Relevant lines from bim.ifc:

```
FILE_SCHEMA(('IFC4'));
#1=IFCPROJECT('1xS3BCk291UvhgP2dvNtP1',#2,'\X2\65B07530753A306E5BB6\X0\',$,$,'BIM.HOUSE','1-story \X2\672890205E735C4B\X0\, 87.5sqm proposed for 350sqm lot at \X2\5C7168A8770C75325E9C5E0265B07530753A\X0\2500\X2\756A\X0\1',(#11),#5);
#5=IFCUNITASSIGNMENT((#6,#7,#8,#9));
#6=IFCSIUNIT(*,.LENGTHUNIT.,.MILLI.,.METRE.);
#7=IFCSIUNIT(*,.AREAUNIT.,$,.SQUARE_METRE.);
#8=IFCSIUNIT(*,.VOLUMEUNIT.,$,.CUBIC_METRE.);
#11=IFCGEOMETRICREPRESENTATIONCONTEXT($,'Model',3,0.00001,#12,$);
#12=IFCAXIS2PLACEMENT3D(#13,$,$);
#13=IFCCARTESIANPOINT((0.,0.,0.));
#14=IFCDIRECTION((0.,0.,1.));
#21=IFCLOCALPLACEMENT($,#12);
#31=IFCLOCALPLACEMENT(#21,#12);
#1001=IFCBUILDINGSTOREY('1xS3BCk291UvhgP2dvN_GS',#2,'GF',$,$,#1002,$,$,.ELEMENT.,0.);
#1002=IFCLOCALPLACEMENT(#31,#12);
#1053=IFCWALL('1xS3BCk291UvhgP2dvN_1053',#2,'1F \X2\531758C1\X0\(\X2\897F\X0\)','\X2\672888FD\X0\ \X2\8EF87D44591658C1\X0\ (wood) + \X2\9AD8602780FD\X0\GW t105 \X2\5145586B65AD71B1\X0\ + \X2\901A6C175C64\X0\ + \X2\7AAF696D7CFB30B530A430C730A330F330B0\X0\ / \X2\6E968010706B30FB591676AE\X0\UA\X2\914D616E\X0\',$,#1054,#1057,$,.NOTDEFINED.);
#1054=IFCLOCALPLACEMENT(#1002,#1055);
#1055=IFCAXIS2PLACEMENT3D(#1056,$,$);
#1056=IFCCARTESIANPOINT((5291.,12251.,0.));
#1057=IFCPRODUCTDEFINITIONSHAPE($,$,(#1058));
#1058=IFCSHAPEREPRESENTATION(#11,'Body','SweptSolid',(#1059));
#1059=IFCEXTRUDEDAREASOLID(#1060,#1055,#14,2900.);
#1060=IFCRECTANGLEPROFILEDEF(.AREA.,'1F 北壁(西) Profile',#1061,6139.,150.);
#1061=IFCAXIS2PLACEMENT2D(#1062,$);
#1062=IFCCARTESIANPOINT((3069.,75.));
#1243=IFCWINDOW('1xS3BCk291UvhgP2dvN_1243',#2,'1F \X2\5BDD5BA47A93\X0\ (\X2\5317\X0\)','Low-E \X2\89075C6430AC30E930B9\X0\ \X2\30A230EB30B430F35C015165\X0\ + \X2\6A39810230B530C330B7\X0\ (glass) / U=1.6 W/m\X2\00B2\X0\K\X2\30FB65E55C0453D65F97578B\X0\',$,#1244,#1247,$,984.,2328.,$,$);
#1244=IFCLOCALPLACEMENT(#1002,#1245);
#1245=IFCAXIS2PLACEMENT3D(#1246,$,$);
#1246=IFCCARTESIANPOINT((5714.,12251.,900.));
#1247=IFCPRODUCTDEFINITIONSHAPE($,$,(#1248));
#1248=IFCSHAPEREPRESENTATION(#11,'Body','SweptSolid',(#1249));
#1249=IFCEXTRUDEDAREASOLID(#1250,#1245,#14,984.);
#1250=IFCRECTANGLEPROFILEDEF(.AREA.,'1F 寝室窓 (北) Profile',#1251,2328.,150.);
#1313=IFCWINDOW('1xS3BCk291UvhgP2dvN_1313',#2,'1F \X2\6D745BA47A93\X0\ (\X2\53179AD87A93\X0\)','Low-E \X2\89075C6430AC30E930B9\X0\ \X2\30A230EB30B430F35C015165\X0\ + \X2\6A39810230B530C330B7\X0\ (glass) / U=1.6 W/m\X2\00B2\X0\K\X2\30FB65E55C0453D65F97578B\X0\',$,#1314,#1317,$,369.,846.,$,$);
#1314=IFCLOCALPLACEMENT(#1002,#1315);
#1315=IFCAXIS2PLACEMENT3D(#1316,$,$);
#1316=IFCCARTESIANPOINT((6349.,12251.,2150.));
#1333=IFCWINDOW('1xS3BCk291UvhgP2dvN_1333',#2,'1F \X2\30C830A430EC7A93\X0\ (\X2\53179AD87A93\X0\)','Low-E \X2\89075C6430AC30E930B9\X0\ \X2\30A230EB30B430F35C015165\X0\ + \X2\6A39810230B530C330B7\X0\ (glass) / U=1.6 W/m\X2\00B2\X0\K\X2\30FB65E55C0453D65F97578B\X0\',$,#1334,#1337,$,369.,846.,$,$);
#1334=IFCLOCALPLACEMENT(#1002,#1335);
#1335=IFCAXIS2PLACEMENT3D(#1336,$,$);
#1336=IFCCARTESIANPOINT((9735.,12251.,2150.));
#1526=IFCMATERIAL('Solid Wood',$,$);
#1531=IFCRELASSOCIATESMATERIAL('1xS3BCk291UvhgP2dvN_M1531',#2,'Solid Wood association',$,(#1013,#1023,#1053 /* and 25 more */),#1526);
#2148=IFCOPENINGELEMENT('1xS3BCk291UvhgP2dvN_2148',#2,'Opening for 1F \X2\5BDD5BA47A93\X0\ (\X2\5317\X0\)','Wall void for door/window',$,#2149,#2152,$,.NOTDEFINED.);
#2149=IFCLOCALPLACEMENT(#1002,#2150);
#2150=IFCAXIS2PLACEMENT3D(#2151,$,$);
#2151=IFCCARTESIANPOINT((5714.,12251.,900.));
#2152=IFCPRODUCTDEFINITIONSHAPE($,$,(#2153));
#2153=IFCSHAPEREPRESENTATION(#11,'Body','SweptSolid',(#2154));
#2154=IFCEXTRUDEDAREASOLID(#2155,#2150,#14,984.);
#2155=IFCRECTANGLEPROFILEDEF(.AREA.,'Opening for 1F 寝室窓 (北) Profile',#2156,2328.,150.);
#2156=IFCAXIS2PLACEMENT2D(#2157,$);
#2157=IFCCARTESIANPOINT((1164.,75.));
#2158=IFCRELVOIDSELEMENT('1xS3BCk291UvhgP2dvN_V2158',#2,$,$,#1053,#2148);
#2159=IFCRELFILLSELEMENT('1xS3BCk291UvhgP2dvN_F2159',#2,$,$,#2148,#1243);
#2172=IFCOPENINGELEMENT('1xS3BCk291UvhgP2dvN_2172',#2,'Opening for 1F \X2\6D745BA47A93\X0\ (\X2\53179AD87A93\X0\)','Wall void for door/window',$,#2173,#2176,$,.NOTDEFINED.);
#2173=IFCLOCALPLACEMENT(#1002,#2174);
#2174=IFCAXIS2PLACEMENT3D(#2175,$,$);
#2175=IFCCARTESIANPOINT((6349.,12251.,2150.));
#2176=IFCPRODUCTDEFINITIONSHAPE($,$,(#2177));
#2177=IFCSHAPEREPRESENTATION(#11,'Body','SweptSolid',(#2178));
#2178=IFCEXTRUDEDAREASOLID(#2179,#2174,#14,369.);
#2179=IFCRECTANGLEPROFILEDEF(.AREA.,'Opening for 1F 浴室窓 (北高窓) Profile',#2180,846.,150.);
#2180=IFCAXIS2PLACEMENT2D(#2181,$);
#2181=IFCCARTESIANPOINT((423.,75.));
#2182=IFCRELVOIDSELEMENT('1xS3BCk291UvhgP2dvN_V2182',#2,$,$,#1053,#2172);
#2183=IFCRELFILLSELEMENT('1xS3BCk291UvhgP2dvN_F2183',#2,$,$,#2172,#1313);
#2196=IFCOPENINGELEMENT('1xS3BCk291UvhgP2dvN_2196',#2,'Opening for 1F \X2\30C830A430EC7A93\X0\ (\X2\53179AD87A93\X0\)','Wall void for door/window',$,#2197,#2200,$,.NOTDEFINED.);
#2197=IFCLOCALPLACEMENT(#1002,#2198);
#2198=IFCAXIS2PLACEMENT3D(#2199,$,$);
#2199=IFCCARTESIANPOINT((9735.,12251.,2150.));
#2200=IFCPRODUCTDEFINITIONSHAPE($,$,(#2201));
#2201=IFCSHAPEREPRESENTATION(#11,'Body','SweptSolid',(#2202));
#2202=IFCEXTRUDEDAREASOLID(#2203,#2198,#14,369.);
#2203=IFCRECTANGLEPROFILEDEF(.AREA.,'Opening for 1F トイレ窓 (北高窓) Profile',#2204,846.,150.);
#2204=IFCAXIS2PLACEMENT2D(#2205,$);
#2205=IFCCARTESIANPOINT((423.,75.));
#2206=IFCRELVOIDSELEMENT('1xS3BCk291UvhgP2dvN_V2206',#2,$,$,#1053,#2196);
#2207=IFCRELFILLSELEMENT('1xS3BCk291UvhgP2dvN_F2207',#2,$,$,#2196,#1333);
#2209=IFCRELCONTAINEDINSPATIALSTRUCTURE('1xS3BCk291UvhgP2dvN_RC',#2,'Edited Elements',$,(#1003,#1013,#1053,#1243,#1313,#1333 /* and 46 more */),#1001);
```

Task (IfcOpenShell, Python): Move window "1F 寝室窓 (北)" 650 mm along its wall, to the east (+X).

```python
import ifcopenshell
import ifcopenshell.api.geometry
import ifcopenshell.util.placement

model = ifcopenshell.open("bim.ifc")

window = model.by_id(1243)
opening = window.FillsVoids[0].RelatingOpeningElement
wall = opening.VoidsElements[0].RelatingBuildingElement

wall_matrix = ifcopenshell.util.placement.get_local_placement(wall.ObjectPlacement)
shift = wall_matrix[:3, 0] * 650.0
before = ifcopenshell.util.placement.get_local_placement(window.ObjectPlacement)[:3, 3].copy()

# The window is not placed relative to its opening, so move both.
for product in (opening, window):
    matrix = ifcopenshell.util.placement.get_local_placement(product.ObjectPlacement)
    matrix[:3, 3] += shift
    ifcopenshell.api.geometry.edit_object_placement(model, product=product, matrix=matrix, is_si=False)

after = ifcopenshell.util.placement.get_local_placement(window.ObjectPlacement)[:3, 3]
print("window moved by", (after - before).round(3) + 0.0)

model.write("bim_updated.ifc")
```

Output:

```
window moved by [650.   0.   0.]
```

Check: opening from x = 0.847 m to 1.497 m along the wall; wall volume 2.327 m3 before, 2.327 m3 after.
